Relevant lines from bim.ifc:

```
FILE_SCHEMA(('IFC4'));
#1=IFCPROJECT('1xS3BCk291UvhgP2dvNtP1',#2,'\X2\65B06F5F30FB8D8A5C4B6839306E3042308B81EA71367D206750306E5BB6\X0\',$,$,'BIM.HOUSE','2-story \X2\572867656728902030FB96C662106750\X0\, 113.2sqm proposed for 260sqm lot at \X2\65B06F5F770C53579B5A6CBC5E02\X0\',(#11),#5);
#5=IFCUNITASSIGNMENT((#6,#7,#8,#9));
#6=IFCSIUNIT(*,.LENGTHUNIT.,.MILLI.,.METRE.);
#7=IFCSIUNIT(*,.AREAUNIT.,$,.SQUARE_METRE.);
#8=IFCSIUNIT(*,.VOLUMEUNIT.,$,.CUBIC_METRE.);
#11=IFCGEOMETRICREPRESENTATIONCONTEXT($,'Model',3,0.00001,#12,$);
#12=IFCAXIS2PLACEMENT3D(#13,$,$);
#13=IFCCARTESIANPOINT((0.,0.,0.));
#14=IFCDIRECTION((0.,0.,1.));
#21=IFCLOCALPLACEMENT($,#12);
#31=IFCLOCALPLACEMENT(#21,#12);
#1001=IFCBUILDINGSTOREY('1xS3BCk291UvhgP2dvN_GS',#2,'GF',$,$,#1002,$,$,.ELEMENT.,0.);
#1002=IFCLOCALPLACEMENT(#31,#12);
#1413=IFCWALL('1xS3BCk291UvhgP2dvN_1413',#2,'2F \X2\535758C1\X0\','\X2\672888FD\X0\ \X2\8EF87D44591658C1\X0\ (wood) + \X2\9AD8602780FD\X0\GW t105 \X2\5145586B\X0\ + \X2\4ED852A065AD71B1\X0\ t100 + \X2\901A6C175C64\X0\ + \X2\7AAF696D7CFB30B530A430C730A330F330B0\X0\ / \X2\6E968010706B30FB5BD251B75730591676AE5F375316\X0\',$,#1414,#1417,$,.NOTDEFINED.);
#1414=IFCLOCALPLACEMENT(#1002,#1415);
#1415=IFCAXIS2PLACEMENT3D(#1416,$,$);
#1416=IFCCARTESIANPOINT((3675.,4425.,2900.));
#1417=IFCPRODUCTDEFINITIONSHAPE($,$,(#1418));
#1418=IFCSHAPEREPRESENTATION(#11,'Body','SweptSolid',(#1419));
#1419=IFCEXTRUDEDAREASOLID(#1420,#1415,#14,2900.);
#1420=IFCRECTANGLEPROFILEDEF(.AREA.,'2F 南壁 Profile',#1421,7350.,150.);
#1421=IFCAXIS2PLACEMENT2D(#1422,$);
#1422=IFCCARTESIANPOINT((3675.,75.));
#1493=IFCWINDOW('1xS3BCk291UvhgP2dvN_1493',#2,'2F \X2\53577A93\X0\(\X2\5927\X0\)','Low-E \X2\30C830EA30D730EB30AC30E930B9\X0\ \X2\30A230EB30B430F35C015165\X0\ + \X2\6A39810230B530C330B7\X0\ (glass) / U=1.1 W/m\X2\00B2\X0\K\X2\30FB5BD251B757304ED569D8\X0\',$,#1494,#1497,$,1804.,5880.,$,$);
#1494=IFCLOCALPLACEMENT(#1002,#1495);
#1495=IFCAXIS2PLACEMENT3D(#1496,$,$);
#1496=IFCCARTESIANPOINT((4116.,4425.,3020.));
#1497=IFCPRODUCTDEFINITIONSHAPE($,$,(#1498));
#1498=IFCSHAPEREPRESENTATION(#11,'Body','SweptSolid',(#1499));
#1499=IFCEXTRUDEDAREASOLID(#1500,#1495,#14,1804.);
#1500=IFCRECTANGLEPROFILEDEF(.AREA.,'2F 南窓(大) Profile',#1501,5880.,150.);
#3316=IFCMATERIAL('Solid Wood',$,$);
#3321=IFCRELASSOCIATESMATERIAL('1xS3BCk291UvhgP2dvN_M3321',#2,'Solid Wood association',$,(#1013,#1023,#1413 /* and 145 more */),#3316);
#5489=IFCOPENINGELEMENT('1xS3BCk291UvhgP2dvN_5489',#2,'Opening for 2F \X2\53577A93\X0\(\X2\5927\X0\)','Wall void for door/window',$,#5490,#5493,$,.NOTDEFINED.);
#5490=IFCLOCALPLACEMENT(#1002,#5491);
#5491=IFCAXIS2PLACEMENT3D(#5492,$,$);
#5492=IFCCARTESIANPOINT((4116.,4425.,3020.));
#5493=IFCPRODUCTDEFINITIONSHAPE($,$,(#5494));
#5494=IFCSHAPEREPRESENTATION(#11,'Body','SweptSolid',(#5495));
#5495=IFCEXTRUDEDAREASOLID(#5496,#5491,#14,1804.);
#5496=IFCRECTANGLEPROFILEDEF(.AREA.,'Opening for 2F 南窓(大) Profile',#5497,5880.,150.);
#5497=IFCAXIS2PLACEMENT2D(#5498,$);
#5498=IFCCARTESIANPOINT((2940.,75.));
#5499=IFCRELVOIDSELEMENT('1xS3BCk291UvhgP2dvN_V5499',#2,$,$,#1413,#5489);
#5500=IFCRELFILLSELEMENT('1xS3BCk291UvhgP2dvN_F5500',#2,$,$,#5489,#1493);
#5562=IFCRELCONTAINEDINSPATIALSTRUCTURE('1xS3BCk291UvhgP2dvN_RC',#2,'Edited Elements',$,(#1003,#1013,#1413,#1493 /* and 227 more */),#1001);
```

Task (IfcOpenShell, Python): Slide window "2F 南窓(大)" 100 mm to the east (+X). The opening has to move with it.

```python
import ifcopenshell
import ifcopenshell.api.geometry
import ifcopenshell.util.placement
import ifcopenshell.util.unit

model = ifcopenshell.open("bim.ifc")
unit_scale = ifcopenshell.util.unit.calculate_unit_scale(model)

window = model.by_guid("1xS3BCk291UvhgP2dvN_1493")
opening = window.FillsVoids[0].RelatingOpeningElement
wall = opening.VoidsElements[0].RelatingBuildingElement

wall_matrix = ifcopenshell.util.placement.get_local_placement(wall.ObjectPlacement)
shift = wall_matrix[:3, 0] * 0.1 / unit_scale
before = ifcopenshell.util.placement.get_local_placement(window.ObjectPlacement)[:3, 3].copy()

# The window is not placed relative to its opening, so move both.
for product in (opening, window):
    matrix = ifcopenshell.util.placement.get_local_placement(product.ObjectPlacement)
    matrix[:3, 3] += shift
    ifcopenshell.api.geometry.edit_object_placement(model, product=product, matrix=matrix, is_si=False)

after = ifcopenshell.util.placement.get_local_placement(window.ObjectPlacement)[:3, 3]
print("window moved by", (after - before).round(3) + 0.0)

model.write("bim-out.ifc")
```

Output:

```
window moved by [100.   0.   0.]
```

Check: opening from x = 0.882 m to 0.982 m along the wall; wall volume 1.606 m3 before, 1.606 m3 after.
